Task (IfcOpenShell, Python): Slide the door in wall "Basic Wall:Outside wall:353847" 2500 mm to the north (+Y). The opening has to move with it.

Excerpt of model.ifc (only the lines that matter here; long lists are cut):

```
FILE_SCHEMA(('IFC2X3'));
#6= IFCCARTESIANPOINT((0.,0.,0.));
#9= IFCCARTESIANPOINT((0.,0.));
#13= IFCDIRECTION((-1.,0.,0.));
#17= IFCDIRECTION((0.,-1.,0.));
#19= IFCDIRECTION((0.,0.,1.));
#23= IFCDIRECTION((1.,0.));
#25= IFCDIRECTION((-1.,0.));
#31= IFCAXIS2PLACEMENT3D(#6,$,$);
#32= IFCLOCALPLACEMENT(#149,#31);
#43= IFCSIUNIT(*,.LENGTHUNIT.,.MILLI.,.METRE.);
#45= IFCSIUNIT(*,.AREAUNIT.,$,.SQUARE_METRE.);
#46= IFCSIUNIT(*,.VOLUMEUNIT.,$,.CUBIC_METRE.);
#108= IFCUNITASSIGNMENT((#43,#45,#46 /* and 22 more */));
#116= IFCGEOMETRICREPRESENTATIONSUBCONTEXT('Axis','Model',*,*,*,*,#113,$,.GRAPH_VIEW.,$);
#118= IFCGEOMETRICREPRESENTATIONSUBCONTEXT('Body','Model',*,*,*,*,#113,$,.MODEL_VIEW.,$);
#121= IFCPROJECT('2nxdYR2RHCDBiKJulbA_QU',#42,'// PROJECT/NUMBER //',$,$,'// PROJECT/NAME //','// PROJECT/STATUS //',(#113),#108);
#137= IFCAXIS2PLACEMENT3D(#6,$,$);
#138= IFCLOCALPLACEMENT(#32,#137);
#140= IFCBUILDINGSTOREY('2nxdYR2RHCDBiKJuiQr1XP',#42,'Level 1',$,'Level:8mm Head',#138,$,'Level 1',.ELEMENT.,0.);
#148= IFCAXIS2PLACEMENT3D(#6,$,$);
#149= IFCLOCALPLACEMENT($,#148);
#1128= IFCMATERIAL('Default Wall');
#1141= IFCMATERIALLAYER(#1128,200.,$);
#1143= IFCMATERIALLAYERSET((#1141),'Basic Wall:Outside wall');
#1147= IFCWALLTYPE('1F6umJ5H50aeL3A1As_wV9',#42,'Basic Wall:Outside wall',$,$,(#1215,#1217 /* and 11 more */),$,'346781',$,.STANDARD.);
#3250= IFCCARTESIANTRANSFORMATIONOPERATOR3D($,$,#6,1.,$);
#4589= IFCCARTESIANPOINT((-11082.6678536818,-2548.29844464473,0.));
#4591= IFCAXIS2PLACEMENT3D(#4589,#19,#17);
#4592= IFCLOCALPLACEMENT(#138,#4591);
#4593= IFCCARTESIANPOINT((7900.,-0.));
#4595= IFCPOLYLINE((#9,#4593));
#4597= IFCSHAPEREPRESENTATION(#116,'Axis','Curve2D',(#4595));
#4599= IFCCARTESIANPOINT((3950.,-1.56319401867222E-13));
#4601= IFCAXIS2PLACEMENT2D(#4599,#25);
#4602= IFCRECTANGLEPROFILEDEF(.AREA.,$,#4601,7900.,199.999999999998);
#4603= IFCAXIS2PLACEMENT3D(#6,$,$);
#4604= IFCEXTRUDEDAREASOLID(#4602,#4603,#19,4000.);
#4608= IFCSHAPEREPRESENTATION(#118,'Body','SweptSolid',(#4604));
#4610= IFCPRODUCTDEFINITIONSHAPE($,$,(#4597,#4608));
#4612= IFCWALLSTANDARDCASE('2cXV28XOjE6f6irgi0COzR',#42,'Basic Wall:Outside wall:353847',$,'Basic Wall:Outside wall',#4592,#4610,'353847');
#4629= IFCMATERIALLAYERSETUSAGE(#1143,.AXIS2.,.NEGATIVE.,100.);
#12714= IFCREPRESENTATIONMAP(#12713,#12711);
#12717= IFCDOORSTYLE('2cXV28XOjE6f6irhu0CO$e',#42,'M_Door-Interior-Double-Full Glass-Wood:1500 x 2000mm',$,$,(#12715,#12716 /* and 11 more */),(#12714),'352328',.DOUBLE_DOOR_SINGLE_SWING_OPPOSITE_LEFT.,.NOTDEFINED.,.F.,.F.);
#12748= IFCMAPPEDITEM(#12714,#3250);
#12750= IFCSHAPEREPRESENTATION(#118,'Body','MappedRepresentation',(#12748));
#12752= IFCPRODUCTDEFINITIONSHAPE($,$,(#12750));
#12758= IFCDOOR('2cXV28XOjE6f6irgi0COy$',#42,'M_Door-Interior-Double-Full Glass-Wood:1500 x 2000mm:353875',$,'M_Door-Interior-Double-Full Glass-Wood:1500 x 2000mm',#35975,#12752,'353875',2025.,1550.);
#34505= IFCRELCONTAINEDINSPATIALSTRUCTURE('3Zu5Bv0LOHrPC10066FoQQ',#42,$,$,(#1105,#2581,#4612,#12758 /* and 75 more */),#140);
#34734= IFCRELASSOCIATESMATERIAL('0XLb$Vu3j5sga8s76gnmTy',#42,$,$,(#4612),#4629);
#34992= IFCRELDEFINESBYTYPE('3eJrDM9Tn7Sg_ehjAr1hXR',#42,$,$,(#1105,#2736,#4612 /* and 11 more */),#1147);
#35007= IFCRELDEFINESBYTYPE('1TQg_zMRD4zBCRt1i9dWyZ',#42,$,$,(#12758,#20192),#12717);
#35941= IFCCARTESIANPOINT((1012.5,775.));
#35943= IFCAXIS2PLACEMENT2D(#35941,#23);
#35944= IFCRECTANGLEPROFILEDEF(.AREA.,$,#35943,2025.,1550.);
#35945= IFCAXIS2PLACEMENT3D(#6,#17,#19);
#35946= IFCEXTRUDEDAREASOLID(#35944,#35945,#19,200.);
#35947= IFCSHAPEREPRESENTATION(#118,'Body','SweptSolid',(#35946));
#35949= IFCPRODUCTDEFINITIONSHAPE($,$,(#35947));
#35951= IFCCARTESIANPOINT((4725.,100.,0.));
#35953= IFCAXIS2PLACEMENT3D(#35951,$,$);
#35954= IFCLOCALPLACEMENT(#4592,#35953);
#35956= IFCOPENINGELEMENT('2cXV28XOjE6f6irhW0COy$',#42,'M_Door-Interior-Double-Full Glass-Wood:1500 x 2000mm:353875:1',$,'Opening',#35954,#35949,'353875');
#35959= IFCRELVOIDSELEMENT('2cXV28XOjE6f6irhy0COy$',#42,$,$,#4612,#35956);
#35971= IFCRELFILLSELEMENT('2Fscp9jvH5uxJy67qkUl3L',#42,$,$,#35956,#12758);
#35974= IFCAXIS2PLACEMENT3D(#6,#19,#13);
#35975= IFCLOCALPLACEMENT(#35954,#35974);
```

```python
import ifcopenshell
import ifcopenshell.api.geometry
import ifcopenshell.util.placement
import ifcopenshell.util.unit

model = ifcopenshell.open("model.ifc")
unit_scale = ifcopenshell.util.unit.calculate_unit_scale(model)

door = model.by_guid("2cXV28XOjE6f6irgi0COy$")
opening = door.FillsVoids[0].RelatingOpeningElement
wall = opening.VoidsElements[0].RelatingBuildingElement

wall_matrix = ifcopenshell.util.placement.get_local_placement(wall.ObjectPlacement)
shift = wall_matrix[:3, 0] * -2.5 / unit_scale
before = ifcopenshell.util.placement.get_local_placement(door.ObjectPlacement)[:3, 3].copy()

# The door is placed relative to its opening, so it follows when the opening moves.
matrix = ifcopenshell.util.placement.get_local_placement(opening.ObjectPlacement)
matrix[:3, 3] += shift
ifcopenshell.api.geometry.edit_object_placement(
    model, product=opening, matrix=matrix, is_si=False, should_transform_children=True
)

after = ifcopenshell.util.placement.get_local_placement(door.ObjectPlacement)[:3, 3]
print("door moved by", (after - before).round(3) + 0.0)

model.write("model_updated.ifc")
```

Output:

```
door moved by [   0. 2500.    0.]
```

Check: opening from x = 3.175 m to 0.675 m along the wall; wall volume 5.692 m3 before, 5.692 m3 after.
